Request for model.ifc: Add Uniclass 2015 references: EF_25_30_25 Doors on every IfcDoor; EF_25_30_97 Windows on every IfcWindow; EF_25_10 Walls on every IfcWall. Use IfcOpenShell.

First a look at what the model holds.

```python
import ifcopenshell

model = ifcopenshell.open("model.ifc")
print(model.schema)
print("classifications:", [c.Name for c in model.by_type("IfcClassification")])
for ifc_class in ("IfcDoor", "IfcRoof", "IfcStair", "IfcWall", "IfcWindow"):
    print(ifc_class, len(model.by_type(ifc_class)))
```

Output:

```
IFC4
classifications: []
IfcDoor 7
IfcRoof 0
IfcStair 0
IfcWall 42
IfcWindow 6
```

```python
import ifcopenshell
import ifcopenshell.api.classification

model = ifcopenshell.open("model.ifc")

system = ifcopenshell.api.classification.add_classification(model, classification="Uniclass 2015")

codes = {
    "IfcDoor": ("EF_25_30_25", "Doors"),
    "IfcWindow": ("EF_25_30_97", "Windows"),
    "IfcWall": ("EF_25_10", "Walls"),
}
for ifc_class, (code, name) in codes.items():
    products = model.by_type(ifc_class)
    ifcopenshell.api.classification.add_reference(
        model, products=products, classification=system, identification=code, name=name
    )
    print(code, len(products))

model.write("model-out.ifc")
```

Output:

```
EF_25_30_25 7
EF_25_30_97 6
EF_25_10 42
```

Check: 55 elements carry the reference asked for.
